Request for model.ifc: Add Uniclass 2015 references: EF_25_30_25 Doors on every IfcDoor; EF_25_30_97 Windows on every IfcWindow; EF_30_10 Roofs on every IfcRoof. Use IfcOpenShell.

First a look at what the model holds.

```python
import ifcopenshell

model = ifcopenshell.open("model.ifc")
print(model.schema)
print("classifications:", [c.Name for c in model.by_type("IfcClassification")])
for ifc_class in ("IfcDoor", "IfcRoof", "IfcStair", "IfcWall", "IfcWindow"):
    print(ifc_class, len(model.by_type(ifc_class)))
```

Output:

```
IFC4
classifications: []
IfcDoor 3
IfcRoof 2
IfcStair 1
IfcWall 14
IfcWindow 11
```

```python
import ifcopenshell
import ifcopenshell.api.classification

model = ifcopenshell.open("model.ifc")

system = ifcopenshell.api.classification.add_classification(model, classification="Uniclass 2015")

codes = {
    "IfcDoor": ("EF_25_30_25", "Doors"),
    "IfcWindow": ("EF_25_30_97", "Windows"),
    "IfcRoof": ("EF_30_10", "Roofs"),
}
for ifc_class, (code, name) in codes.items():
    products = model.by_type(ifc_class)
    ifcopenshell.api.classification.add_reference(
        model, products=products, classification=system, identification=code, name=name
    )
    print(code, len(products))

model.write("model-out.ifc")
```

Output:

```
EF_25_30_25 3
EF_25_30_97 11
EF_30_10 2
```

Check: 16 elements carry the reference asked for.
